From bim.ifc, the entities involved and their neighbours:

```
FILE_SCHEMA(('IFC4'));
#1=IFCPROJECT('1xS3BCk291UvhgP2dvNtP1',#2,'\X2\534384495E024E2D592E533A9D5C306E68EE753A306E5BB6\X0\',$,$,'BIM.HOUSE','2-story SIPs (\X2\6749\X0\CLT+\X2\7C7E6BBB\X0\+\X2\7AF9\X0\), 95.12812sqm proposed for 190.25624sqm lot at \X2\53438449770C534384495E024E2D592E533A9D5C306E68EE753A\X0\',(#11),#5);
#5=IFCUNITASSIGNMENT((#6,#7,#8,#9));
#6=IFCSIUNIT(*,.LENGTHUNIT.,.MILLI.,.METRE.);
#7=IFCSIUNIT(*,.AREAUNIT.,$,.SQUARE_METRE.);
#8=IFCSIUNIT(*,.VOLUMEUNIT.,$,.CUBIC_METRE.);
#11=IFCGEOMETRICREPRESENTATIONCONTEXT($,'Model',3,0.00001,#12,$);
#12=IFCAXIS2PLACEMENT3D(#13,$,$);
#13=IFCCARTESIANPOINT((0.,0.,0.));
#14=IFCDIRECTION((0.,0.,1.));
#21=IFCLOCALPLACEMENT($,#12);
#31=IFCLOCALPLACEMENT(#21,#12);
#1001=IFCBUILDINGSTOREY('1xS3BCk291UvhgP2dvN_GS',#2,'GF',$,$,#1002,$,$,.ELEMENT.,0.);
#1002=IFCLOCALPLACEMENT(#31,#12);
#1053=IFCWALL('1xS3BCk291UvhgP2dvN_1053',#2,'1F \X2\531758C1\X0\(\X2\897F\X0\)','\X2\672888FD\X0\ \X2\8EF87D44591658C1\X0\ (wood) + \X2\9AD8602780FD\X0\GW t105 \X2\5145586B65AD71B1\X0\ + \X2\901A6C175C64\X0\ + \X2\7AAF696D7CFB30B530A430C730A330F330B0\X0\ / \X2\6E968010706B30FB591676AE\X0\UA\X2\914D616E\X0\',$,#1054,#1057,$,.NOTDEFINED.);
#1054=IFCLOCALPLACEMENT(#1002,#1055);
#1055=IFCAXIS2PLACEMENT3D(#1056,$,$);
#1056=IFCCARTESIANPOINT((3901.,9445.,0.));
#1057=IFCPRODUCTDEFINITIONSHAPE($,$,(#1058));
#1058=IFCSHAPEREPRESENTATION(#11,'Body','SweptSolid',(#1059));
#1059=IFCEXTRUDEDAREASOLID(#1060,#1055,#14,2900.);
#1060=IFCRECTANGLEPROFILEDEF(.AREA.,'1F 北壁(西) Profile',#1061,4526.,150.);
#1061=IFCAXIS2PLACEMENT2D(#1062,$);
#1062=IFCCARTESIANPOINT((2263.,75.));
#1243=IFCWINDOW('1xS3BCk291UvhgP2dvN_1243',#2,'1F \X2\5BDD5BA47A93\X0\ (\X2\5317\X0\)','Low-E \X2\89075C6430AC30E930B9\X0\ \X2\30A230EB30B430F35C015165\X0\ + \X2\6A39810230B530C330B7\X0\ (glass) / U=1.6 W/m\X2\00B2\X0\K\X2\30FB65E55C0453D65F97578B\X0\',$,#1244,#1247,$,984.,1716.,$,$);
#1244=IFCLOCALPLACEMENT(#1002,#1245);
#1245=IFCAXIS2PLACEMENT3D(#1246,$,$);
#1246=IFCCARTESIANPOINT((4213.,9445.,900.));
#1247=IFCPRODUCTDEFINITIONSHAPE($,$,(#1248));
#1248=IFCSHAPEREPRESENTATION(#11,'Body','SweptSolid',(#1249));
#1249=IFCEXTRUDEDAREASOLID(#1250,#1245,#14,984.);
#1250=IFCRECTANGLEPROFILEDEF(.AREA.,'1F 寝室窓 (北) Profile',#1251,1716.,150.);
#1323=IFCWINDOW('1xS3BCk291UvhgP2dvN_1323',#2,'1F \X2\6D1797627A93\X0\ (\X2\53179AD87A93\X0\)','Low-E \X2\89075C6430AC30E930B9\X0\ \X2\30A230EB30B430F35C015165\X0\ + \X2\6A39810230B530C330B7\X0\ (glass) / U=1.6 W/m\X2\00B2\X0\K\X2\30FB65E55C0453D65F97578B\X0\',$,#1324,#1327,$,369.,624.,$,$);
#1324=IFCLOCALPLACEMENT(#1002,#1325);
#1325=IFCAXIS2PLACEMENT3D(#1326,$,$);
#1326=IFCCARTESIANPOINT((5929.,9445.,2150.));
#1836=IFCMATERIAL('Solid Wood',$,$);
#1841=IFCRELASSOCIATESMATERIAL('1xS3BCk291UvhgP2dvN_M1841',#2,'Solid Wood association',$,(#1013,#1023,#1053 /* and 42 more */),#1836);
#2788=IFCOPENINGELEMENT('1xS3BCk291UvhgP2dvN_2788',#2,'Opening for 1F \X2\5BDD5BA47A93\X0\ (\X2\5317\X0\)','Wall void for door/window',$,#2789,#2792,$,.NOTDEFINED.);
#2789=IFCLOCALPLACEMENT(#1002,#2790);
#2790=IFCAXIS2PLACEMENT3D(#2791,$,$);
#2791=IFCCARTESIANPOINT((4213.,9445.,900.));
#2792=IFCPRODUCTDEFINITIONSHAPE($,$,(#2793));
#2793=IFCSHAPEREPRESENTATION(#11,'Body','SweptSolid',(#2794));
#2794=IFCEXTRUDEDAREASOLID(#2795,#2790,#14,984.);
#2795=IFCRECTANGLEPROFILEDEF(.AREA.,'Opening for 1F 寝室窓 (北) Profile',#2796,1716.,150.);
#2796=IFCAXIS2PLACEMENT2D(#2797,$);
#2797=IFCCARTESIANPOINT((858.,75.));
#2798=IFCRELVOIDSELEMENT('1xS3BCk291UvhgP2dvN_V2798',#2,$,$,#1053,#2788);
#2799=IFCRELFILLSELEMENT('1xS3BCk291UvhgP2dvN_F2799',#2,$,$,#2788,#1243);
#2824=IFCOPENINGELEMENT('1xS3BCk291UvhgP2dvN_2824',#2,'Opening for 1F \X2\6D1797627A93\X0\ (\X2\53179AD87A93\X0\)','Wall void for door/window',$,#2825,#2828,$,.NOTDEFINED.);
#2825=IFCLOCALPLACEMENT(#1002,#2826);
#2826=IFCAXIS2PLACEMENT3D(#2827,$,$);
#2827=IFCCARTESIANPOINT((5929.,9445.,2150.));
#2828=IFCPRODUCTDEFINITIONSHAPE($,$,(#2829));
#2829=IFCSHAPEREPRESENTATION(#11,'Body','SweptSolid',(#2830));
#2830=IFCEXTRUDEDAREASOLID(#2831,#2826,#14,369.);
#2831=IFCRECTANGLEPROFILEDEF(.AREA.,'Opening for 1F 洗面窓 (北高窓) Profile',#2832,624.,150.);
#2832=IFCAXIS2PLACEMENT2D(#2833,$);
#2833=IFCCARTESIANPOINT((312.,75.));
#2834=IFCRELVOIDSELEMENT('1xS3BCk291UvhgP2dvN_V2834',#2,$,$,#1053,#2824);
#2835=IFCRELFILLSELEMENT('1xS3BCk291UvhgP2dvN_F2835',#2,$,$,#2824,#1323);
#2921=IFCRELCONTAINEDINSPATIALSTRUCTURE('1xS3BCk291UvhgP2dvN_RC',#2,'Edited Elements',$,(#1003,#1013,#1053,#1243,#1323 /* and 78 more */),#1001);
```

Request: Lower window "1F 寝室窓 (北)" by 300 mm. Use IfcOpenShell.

```python
import numpy as np
import ifcopenshell
import ifcopenshell.api.geometry
import ifcopenshell.util.placement
import ifcopenshell.util.unit

model = ifcopenshell.open("bim.ifc")
unit_scale = ifcopenshell.util.unit.calculate_unit_scale(model)

window = model.by_guid("1xS3BCk291UvhgP2dvN_1243")
opening = window.FillsVoids[0].RelatingOpeningElement
dz = -0.3 / unit_scale

shift = np.array([0.0, 0.0, dz])
# The window is not placed relative to its opening, so move both.
for product in (opening, window):
    matrix = ifcopenshell.util.placement.get_local_placement(product.ObjectPlacement)
    matrix[:3, 3] += shift
    ifcopenshell.api.geometry.edit_object_placement(model, product=product, matrix=matrix, is_si=False)

print(f"moved by {dz * unit_scale:+.3f} m")

model.write("bim_edited.ifc")
```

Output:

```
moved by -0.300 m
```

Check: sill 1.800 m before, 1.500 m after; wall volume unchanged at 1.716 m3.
